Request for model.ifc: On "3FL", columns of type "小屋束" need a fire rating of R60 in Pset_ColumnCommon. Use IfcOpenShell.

First a look at what the model holds.

```python
import ifcopenshell
import ifcopenshell.util.element

model = ifcopenshell.open("model.ifc")
print(model.schema)
storey = next(s for s in model.by_type("IfcBuildingStorey") if s.Name == "3FL")
columns = [e for e in ifcopenshell.util.element.get_decomposition(storey) if e.is_a("IfcColumn")]
seen = {}
for e in columns:
    element_type = ifcopenshell.util.element.get_type(e)
    key = (element_type.Name if element_type != e and element_type else None, ifcopenshell.util.element.get_pset(e, "Pset_ColumnCommon", "FireRating"))
    seen[key] = seen.get(key, 0) + 1
for (name, value), count in sorted(seen.items(), key=str):
    print(count, "x", name, "|", value)
```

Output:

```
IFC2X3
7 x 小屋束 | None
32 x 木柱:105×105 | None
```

```python
import ifcopenshell
import ifcopenshell.api.pset
import ifcopenshell.util.element

model = ifcopenshell.open("model.ifc")

storey = next(s for s in model.by_type("IfcBuildingStorey") if s.Name == "3FL")
columns = [e for e in ifcopenshell.util.element.get_decomposition(storey) if e.is_a("IfcColumn")]

count = 0
for e in columns:
    element_type = ifcopenshell.util.element.get_type(e)
    if element_type in (None, e) or element_type.Name != "小屋束":
        continue
    # add_pset returns the element's existing set when there is one.
    pset = ifcopenshell.api.pset.add_pset(model, product=e, name="Pset_ColumnCommon")
    ifcopenshell.api.pset.edit_pset(model, pset=pset, properties={"FireRating": "R60"})
    count += 1

print(count, "columns updated")

model.write("model_updated.ifc")
```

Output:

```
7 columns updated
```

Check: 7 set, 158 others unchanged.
